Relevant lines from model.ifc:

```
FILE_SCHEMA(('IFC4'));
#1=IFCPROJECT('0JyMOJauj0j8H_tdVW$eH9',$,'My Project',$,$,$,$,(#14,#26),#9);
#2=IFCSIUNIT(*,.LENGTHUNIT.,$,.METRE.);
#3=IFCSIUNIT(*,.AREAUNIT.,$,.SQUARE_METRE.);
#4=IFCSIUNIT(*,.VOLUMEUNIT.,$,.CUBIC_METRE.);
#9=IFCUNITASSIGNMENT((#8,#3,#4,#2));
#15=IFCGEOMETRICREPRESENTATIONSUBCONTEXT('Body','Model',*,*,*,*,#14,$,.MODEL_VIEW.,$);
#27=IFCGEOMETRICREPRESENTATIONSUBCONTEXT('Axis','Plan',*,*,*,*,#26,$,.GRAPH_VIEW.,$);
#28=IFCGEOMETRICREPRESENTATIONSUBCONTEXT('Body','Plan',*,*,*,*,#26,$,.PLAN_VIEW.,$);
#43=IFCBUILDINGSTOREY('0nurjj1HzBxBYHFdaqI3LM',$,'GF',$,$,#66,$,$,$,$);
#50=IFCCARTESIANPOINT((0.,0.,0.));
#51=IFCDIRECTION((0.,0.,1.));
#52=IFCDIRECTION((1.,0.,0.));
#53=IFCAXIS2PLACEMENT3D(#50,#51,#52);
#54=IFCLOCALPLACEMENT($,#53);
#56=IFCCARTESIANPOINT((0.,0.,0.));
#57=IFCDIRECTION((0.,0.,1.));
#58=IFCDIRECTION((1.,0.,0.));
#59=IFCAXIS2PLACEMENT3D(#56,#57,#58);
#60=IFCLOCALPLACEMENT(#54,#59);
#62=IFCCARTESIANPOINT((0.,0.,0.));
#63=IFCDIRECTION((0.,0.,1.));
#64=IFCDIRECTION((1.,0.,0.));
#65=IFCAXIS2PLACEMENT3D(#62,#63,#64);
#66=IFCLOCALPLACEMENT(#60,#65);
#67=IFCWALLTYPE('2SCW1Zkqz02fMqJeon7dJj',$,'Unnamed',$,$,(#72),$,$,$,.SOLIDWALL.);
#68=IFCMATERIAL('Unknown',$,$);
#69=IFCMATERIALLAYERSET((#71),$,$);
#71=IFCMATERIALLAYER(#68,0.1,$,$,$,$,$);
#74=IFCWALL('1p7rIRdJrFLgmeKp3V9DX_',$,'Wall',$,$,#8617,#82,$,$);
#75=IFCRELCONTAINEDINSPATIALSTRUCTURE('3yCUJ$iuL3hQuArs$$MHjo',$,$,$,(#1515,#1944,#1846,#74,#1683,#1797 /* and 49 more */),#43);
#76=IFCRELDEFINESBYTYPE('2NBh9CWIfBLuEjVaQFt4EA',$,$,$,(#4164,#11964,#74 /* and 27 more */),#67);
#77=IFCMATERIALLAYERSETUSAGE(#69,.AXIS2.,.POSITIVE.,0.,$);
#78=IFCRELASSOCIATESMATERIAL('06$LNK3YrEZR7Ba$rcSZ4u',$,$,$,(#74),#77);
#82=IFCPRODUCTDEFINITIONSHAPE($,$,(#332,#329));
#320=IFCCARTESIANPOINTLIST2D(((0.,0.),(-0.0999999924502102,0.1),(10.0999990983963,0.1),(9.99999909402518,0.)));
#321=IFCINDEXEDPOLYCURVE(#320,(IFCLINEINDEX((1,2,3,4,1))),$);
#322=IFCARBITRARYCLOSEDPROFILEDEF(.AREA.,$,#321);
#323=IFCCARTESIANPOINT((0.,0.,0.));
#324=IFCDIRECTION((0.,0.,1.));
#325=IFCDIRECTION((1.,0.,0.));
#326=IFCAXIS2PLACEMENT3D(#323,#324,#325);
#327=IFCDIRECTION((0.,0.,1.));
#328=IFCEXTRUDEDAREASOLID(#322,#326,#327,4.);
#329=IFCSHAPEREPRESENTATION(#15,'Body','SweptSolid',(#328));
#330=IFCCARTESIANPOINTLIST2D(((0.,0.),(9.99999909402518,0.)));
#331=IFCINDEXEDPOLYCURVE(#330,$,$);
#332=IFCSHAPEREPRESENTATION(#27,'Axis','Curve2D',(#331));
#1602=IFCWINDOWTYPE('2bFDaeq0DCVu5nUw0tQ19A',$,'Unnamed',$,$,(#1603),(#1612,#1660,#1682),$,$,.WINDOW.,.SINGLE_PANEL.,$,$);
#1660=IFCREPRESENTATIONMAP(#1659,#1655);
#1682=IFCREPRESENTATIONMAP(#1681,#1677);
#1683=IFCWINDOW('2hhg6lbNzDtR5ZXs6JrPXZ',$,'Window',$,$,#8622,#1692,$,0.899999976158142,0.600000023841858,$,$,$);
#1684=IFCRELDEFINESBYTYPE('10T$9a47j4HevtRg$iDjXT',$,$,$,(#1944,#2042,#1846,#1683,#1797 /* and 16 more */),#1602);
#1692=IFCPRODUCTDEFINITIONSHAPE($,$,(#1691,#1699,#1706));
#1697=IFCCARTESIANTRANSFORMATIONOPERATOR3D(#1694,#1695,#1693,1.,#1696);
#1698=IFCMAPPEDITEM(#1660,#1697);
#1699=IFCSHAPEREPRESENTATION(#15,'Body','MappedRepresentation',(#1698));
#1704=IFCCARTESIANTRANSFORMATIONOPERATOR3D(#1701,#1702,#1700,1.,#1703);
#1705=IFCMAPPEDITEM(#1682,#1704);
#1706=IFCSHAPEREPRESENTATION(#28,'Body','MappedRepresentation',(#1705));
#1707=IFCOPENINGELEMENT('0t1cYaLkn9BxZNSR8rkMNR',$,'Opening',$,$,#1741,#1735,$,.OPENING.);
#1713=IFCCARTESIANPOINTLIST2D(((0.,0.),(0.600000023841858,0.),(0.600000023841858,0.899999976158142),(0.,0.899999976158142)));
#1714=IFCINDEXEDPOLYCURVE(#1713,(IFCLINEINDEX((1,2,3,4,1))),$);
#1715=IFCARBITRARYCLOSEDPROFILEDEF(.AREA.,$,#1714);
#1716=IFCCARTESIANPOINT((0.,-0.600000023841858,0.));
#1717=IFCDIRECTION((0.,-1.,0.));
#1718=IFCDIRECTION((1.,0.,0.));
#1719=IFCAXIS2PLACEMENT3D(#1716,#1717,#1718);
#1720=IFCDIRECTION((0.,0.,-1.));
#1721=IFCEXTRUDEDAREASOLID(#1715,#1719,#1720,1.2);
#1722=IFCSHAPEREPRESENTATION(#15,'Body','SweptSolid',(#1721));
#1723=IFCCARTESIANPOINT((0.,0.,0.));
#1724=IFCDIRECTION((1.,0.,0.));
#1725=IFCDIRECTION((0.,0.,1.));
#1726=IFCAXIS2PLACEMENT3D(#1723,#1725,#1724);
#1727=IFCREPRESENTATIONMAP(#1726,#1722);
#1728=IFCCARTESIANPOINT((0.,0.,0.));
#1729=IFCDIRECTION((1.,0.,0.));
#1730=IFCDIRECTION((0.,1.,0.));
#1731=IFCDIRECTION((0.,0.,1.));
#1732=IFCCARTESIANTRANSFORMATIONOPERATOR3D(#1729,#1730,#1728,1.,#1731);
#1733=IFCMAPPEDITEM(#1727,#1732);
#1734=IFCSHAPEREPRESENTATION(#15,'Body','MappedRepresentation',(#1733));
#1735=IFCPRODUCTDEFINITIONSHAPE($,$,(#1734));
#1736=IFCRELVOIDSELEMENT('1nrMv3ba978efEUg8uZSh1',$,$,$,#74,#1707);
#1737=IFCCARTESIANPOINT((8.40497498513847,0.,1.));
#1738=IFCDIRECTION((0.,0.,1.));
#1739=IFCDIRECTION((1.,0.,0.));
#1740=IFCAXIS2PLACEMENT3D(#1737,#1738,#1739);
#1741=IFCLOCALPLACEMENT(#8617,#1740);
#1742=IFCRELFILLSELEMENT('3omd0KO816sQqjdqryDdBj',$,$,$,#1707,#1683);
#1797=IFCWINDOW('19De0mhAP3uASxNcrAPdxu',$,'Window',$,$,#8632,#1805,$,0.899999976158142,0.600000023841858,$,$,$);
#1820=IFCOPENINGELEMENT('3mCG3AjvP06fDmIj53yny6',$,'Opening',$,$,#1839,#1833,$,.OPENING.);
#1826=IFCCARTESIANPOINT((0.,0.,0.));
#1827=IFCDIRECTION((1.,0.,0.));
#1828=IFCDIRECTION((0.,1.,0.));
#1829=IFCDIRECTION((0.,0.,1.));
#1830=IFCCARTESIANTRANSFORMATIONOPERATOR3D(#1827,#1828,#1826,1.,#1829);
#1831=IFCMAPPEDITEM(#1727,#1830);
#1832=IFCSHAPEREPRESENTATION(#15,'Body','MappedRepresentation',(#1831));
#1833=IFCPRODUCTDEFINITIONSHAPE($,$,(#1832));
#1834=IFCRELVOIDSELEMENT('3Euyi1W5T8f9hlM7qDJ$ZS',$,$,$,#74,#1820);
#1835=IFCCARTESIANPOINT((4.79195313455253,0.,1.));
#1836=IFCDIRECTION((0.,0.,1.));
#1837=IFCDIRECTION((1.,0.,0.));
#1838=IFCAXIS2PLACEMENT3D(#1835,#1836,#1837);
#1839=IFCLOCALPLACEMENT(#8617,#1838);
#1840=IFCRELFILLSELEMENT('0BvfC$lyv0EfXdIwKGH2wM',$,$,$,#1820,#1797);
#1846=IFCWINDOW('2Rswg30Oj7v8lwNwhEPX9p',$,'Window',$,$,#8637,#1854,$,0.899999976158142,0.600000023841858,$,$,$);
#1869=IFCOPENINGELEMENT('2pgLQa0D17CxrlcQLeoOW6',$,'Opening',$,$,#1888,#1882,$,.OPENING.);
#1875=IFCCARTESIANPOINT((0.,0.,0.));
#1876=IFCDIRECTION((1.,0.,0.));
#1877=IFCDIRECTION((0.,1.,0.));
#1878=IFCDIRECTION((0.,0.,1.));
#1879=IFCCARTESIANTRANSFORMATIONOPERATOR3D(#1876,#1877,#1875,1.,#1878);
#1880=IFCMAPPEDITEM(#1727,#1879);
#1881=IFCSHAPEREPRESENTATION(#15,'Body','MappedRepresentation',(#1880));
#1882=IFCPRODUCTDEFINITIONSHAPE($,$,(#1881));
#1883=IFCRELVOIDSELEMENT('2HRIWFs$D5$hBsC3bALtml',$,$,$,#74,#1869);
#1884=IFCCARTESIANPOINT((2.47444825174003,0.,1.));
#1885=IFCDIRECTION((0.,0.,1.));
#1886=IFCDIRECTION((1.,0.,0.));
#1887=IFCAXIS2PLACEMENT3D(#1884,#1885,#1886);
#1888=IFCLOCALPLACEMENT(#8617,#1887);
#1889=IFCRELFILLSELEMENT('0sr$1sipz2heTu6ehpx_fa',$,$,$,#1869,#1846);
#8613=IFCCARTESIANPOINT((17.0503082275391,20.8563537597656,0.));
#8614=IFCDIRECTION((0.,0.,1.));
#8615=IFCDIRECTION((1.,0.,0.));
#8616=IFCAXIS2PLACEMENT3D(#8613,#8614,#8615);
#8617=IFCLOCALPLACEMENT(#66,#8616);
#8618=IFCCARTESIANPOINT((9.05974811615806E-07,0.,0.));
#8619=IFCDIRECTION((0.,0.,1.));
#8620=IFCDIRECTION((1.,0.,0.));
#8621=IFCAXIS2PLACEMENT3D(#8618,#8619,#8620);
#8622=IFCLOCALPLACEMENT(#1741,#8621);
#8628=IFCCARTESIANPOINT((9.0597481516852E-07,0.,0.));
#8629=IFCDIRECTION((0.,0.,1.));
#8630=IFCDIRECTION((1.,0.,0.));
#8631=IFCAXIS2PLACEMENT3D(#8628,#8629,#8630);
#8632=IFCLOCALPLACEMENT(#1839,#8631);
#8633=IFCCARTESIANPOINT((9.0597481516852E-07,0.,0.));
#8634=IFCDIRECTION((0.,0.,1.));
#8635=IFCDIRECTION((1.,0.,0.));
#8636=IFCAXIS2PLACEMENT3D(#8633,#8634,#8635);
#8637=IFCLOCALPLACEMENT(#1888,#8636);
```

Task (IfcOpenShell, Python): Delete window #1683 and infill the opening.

```python
import ifcopenshell
import ifcopenshell.api.feature
import ifcopenshell.api.root
import ifcopenshell.geom
import ifcopenshell.util.shape

model = ifcopenshell.open("model.ifc")
settings = ifcopenshell.geom.settings()


def volume(element):
    """Net volume in cubic metres, openings subtracted."""
    shape = ifcopenshell.geom.create_shape(settings, element)
    return ifcopenshell.util.shape.get_volume(shape.geometry)


window = model.by_id(1683)
opening = window.FillsVoids[0].RelatingOpeningElement
wall = opening.VoidsElements[0].RelatingBuildingElement
before = volume(wall)

ifcopenshell.api.root.remove_product(model, product=window)
ifcopenshell.api.feature.remove_feature(model, feature=opening)

after = volume(wall)

print(f"wall volume {before:.3f} -> {after:.3f} m3")

model.write("model_v2.ifc")
```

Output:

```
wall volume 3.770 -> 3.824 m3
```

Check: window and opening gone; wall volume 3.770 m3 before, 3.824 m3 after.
